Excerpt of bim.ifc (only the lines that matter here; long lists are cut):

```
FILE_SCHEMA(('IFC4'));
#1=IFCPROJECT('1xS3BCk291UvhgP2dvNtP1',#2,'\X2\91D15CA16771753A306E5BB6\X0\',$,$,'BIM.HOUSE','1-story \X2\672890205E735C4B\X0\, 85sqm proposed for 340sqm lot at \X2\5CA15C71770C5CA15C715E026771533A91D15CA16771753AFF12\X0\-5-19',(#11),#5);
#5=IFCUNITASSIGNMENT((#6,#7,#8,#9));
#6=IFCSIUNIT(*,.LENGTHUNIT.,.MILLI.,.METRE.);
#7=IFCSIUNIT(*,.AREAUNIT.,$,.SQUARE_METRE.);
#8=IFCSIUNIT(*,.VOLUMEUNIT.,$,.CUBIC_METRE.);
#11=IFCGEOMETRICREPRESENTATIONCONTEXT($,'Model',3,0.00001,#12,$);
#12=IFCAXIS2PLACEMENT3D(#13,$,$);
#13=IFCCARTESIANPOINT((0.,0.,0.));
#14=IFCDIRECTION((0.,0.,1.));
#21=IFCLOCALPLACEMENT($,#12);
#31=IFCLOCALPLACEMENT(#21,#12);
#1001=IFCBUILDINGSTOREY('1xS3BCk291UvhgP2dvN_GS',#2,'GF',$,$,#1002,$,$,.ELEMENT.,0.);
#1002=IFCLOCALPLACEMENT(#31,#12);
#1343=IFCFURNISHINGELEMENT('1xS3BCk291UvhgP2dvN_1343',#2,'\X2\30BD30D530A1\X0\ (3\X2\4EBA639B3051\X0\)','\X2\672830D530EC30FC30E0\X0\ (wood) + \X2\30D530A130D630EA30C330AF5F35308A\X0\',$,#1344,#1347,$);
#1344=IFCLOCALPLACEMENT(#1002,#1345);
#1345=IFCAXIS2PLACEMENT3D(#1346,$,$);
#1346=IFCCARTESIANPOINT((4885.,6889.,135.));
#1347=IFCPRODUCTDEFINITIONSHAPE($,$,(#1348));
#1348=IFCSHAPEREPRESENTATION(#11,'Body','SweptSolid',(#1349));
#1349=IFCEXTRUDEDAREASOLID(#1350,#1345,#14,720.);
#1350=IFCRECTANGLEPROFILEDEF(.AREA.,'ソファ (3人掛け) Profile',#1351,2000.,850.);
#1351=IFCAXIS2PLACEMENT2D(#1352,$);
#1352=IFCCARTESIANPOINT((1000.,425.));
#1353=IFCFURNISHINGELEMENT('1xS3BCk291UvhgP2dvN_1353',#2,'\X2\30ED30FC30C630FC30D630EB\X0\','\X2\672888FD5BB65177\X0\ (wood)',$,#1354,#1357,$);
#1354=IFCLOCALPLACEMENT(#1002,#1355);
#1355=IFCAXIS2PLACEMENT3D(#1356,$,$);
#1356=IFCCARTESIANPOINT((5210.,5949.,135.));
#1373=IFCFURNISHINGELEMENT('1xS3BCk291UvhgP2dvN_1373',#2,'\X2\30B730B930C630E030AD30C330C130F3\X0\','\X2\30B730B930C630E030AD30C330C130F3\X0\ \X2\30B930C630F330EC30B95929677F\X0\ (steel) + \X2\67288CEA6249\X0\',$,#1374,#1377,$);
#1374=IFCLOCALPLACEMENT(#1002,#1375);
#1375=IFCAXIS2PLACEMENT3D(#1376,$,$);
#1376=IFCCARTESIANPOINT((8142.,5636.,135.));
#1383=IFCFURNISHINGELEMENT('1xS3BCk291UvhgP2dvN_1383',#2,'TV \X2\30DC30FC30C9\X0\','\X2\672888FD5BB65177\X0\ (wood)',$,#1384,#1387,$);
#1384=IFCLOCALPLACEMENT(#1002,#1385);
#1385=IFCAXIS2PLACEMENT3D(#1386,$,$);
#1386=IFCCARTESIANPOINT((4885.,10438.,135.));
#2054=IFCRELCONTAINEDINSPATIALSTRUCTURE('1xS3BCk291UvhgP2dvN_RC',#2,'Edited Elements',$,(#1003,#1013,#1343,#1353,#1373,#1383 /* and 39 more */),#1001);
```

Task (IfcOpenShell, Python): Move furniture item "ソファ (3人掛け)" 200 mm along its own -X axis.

```python
import ifcopenshell
import ifcopenshell.api.geometry
import ifcopenshell.util.placement

model = ifcopenshell.open("bim.ifc")

item = model.by_guid("1xS3BCk291UvhgP2dvN_1343")
matrix = ifcopenshell.util.placement.get_local_placement(item.ObjectPlacement)
matrix[:3, 3] -= matrix[:3, 0] * 200.0
ifcopenshell.api.geometry.edit_object_placement(model, product=item, matrix=matrix, is_si=False)

print(ifcopenshell.util.placement.get_local_placement(item.ObjectPlacement).round(3) + 0.0)

model.write("bim_updated.ifc")
```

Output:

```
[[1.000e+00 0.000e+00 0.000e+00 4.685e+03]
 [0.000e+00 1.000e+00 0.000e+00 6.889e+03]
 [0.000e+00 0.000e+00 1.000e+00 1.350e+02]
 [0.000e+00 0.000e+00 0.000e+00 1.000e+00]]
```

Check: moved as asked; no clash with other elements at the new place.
